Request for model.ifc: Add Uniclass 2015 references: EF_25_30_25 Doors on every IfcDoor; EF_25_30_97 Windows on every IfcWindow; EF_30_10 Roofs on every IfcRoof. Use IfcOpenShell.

First a look at what the model holds.

```python
import ifcopenshell

model = ifcopenshell.open("model.ifc")
print(model.schema)
print("classifications:", [c.Name for c in model.by_type("IfcClassification")])
for ifc_class in ("IfcDoor", "IfcRoof", "IfcStair", "IfcWall", "IfcWindow"):
    print(ifc_class, len(model.by_type(ifc_class)))
```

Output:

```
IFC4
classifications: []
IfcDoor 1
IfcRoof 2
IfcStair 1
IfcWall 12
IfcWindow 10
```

```python
import ifcopenshell
import ifcopenshell.api.classification

model = ifcopenshell.open("model.ifc")

system = ifcopenshell.api.classification.add_classification(model, classification="Uniclass 2015")

codes = {
    "IfcDoor": ("EF_25_30_25", "Doors"),
    "IfcWindow": ("EF_25_30_97", "Windows"),
    "IfcRoof": ("EF_30_10", "Roofs"),
}
for ifc_class, (code, name) in codes.items():
    products = model.by_type(ifc_class)
    ifcopenshell.api.classification.add_reference(
        model, products=products, classification=system, identification=code, name=name
    )
    print(code, len(products))

model.write("model_v2.ifc")
```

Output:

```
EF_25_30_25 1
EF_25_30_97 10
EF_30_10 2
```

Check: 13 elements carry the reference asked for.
